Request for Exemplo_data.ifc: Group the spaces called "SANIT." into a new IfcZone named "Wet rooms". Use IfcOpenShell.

First a look at what the model holds.

```python
import ifcopenshell

model = ifcopenshell.open("Exemplo_data.ifc")
print(model.schema)
seen = {}
for space in model.by_type("IfcSpace"):
    seen[space.LongName] = seen.get(space.LongName, 0) + 1
for name, count in sorted(seen.items(), key=str):
    print(count, "x", name)
print("zones:", [z.Name for z in model.by_type("IfcZone")][:20])
```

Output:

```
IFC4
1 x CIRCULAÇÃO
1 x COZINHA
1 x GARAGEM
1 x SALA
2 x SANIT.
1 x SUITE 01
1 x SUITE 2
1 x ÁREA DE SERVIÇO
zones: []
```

```python
import ifcopenshell
import ifcopenshell.api.group
import ifcopenshell.api.root

model = ifcopenshell.open("Exemplo_data.ifc")

names = {"SANIT."}
spaces = [s for s in model.by_type("IfcSpace") if s.LongName in names]

zone = ifcopenshell.api.root.create_entity(model, ifc_class="IfcZone", name="Wet rooms")
ifcopenshell.api.group.assign_group(model, products=spaces, group=zone)
print(len(spaces), "spaces in", zone.Name)

model.write("Exemplo_data-out.ifc")
```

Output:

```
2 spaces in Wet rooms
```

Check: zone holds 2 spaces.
